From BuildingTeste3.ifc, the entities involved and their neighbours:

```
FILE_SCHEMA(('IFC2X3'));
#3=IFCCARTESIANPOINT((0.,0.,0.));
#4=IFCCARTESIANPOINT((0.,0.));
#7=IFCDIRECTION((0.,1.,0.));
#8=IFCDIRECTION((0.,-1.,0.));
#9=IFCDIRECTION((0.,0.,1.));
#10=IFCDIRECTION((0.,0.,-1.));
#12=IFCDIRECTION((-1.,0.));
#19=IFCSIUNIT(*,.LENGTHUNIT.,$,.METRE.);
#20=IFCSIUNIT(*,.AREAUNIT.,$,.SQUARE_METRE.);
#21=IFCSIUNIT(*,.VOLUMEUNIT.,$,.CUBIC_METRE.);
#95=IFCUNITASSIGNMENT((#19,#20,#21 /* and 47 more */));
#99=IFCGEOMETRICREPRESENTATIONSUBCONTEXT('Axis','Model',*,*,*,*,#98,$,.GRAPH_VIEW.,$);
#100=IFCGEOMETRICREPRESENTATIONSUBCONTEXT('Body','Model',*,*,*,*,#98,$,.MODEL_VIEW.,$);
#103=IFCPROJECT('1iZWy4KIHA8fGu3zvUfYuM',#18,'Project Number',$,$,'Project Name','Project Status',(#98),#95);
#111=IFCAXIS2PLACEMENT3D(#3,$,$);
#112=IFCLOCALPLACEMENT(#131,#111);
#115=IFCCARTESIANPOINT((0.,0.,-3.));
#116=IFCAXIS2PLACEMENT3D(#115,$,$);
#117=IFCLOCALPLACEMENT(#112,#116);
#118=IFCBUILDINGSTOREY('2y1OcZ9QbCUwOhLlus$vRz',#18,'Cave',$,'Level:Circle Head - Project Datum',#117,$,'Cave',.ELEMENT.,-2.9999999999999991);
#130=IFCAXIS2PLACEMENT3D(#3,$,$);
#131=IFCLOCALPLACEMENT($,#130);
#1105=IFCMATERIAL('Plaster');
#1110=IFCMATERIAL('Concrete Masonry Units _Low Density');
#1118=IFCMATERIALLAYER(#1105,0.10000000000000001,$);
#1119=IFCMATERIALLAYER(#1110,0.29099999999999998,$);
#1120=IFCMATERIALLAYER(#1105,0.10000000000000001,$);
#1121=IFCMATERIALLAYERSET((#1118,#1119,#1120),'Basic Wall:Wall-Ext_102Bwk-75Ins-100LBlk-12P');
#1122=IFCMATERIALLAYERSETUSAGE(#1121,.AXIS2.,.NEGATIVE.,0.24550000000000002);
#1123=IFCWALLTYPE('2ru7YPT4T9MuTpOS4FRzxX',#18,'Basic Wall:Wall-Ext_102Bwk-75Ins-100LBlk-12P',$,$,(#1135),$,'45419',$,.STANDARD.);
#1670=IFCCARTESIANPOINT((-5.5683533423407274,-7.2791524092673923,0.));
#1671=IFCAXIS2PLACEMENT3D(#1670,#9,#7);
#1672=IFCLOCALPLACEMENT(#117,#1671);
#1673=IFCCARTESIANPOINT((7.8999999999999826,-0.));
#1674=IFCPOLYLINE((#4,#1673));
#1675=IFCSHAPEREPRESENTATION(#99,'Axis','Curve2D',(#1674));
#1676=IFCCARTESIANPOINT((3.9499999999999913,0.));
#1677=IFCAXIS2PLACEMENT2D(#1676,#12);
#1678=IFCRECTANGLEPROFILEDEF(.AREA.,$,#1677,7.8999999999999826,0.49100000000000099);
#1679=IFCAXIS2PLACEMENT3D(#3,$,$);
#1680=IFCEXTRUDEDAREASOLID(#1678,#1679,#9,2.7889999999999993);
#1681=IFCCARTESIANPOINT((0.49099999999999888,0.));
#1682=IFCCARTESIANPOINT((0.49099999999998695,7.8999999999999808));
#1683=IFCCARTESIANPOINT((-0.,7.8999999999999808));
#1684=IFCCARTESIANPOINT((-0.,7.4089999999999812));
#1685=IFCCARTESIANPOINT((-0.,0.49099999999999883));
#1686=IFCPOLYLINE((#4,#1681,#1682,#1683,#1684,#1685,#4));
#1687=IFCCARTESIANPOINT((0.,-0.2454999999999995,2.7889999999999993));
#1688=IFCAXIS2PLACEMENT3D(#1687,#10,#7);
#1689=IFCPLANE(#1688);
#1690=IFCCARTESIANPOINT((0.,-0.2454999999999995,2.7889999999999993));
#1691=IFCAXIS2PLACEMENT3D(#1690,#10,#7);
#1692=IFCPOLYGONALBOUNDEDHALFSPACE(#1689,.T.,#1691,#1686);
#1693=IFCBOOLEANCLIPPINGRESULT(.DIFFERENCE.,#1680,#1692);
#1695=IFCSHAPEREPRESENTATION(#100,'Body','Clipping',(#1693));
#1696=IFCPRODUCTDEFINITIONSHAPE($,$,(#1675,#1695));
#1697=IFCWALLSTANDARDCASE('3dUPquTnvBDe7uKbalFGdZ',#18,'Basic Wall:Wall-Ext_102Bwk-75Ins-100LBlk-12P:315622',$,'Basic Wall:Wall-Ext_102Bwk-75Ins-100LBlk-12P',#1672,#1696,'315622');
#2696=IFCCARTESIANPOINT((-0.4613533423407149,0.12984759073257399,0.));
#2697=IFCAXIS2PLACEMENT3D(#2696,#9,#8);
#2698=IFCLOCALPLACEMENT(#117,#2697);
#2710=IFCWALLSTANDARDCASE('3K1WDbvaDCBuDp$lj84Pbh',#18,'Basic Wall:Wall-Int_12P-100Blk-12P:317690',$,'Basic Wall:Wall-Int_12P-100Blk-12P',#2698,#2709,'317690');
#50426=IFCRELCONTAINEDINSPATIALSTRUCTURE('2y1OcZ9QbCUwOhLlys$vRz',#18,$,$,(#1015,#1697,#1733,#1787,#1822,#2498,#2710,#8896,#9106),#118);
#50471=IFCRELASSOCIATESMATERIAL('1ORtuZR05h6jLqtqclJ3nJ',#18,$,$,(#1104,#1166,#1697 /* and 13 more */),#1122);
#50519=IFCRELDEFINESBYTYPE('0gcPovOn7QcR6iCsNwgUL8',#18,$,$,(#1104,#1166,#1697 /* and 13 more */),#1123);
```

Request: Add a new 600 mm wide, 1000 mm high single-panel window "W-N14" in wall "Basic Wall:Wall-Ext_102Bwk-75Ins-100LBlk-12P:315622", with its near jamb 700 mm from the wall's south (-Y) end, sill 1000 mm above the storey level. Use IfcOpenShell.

```python
import numpy as np
import ifcopenshell
import ifcopenshell.api.feature
import ifcopenshell.api.geometry
import ifcopenshell.api.root
import ifcopenshell.api.spatial
import ifcopenshell.api.type
import ifcopenshell.geom
import ifcopenshell.util.element
import ifcopenshell.util.placement
import ifcopenshell.util.representation
import ifcopenshell.util.shape
import ifcopenshell.util.unit

model = ifcopenshell.open("BuildingTeste3.ifc")
unit_scale = ifcopenshell.util.unit.calculate_unit_scale(model)
settings = ifcopenshell.geom.settings()


def volume(element):
    """Net volume in cubic metres, openings subtracted."""
    shape = ifcopenshell.geom.create_shape(settings, element)
    return ifcopenshell.util.shape.get_volume(shape.geometry)


wall = model.by_guid("3dUPquTnvBDe7uKbalFGdZ")
storey = ifcopenshell.util.element.get_container(wall, ifc_class="IfcBuildingStorey")
context = ifcopenshell.util.representation.get_context(model, "Model", "Body", "MODEL_VIEW")
before = volume(wall)

width, height, from_end, sill = 0.6, 1, 0.7, 1  # metres

# The wall runs along its own X axis, and the end named is its -X end.
wall_shape = ifcopenshell.geom.create_shape(settings, wall)
x, y, z = ifcopenshell.util.shape.get_vertices(wall_shape.geometry).T
start = x.min() + from_end
face, thickness = float(y.min()), float(y.max() - y.min())
wall_matrix = ifcopenshell.util.placement.get_local_placement(wall.ObjectPlacement)
level = ifcopenshell.util.placement.get_local_placement(storey.ObjectPlacement)[2, 3]


def in_wall(x, y):
    """Placement at x, y metres in the wall's axes, at sill height."""
    matrix = wall_matrix.copy()
    matrix[:, 3] = wall_matrix @ np.array([x / unit_scale, y / unit_scale, 0.0, 1.0])
    matrix[2, 3] = level + sill / unit_scale
    return matrix


# Opening: a box that overshoots both wall faces by 50 mm.
opening = ifcopenshell.api.root.create_entity(model, ifc_class="IfcOpeningElement")
box = ifcopenshell.api.geometry.add_wall_representation(
    model, context=context, length=width, height=height, thickness=thickness + 0.1
)
ifcopenshell.api.geometry.assign_representation(model, product=opening, representation=box)
ifcopenshell.api.geometry.edit_object_placement(model, product=opening, matrix=in_wall(start, face - 0.05), is_si=False)
ifcopenshell.api.feature.add_feature(model, feature=opening, element=wall)

window = ifcopenshell.api.root.create_entity(model, ifc_class="IfcWindow", name="W-N14")
window.OverallWidth, window.OverallHeight = width / unit_scale, height / unit_scale
body = ifcopenshell.api.geometry.add_window_representation(
    model,
    context=context,
    overall_width=window.OverallWidth,
    overall_height=window.OverallHeight,
    partition_type="SINGLE_PANEL",
)
ifcopenshell.api.geometry.assign_representation(model, product=window, representation=body)
ifcopenshell.api.spatial.assign_container(model, products=[window], relating_structure=storey)
fills = ifcopenshell.api.feature.add_filling(model, opening=opening, element=window)
fills.OwnerHistory = window.OwnerHistory  # required in IFC2X3

# IFC2X3 keeps the operation on the window style.
style = ifcopenshell.api.root.create_entity(model, ifc_class="IfcWindowStyle", name="W-N14")
style.OperationType, style.ConstructionType = "SINGLE_PANEL", "NOTDEFINED"
style.ParameterTakesPrecedence = style.Sizeable = False
ifcopenshell.api.type.assign_type(model, related_objects=[window], relating_type=style)

# Centre the window in the wall's thickness.
ifcopenshell.api.geometry.edit_object_placement(model, product=window, matrix=in_wall(start, face), is_si=False)
window_shape = ifcopenshell.geom.create_shape(settings, window)
depth = ifcopenshell.util.shape.get_vertices(window_shape.geometry)[:, 1]
offset = face + thickness / 2 - (depth.min() + depth.max()) / 2
ifcopenshell.api.geometry.edit_object_placement(model, product=window, matrix=in_wall(start, offset), is_si=False)

after = volume(wall)

print(f"wall volume {before:.3f} -> {after:.3f} m3")

model.write("BuildingTeste3_edited.ifc")
```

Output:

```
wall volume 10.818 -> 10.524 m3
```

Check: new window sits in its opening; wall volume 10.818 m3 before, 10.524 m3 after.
